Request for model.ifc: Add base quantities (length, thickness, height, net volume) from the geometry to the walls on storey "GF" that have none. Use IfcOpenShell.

First a look at what the model holds.

```python
import ifcopenshell
import ifcopenshell.util.element
import ifcopenshell.util.unit

model = ifcopenshell.open("model.ifc")
print(model.schema)
for unit_type in ("LENGTHUNIT", "AREAUNIT", "VOLUMEUNIT"):
    print(unit_type, ifcopenshell.util.unit.calculate_unit_scale(model, unit_type))
storey = next(s for s in model.by_type("IfcBuildingStorey") if s.Name == "GF")
walls = [e for e in ifcopenshell.util.element.get_decomposition(storey) if e.is_a("IfcWall")]
for e in sorted(walls, key=lambda e: e.id()):
    print(e.id(), e.is_a(), e.Name, list(ifcopenshell.util.element.get_psets(e, qtos_only=True)), sep=" | ")
```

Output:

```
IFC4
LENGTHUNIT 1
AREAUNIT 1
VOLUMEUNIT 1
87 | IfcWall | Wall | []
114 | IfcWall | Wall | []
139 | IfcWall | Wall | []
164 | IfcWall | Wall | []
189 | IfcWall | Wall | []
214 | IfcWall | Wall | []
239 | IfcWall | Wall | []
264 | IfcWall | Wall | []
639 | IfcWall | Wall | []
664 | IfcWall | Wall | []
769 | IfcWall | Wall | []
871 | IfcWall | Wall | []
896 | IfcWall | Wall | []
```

```python
import ifcopenshell
import ifcopenshell.api.pset
import ifcopenshell.geom
import ifcopenshell.util.element
import ifcopenshell.util.shape
import ifcopenshell.util.unit

model = ifcopenshell.open("model.ifc")
unit_scale = ifcopenshell.util.unit.calculate_unit_scale(model)
volume_scale = ifcopenshell.util.unit.calculate_unit_scale(model, "VOLUMEUNIT")
settings = ifcopenshell.geom.settings()

storey = next(s for s in model.by_type("IfcBuildingStorey") if s.Name == "GF")
walls = [e for e in ifcopenshell.util.element.get_decomposition(storey) if e.is_a("IfcWall")]

for e in sorted(walls, key=lambda e: e.id()):
    if ifcopenshell.util.element.get_psets(e, qtos_only=True, should_inherit=False):
        continue
    # Geometry comes back in metres, in the element's own axes.
    shape = ifcopenshell.geom.create_shape(settings, e)
    values = {
        "Length": ifcopenshell.util.shape.get_x(shape.geometry) / unit_scale,
        "Width": ifcopenshell.util.shape.get_y(shape.geometry) / unit_scale,
        "Height": ifcopenshell.util.shape.get_z(shape.geometry) / unit_scale,
        "NetVolume": ifcopenshell.util.shape.get_volume(shape.geometry) / volume_scale,
    }
    qto = ifcopenshell.api.pset.add_qto(model, product=e, name="Qto_WallBaseQuantities")
    ifcopenshell.api.pset.edit_qto(model, qto=qto, properties=values)
    print(e.id(), {k: round(v, 3) for k, v in values.items()})

model.write("model_v2.ifc")
```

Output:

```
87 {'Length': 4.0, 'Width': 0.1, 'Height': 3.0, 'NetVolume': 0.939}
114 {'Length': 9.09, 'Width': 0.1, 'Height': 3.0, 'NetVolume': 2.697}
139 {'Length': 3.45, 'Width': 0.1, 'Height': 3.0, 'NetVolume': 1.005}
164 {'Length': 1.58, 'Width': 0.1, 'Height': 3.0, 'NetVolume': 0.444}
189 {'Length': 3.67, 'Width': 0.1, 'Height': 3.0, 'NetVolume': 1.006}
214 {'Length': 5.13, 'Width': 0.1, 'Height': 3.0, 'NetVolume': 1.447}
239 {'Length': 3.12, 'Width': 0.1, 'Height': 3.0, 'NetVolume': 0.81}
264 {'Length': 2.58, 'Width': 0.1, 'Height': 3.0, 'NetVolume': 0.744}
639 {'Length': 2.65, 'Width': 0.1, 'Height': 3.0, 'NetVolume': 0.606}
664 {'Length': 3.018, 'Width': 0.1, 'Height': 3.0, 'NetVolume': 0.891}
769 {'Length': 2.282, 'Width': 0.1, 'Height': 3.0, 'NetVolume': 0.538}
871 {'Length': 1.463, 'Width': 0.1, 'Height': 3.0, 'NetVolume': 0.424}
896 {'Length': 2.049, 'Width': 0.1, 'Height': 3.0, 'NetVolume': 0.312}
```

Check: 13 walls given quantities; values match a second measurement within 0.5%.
